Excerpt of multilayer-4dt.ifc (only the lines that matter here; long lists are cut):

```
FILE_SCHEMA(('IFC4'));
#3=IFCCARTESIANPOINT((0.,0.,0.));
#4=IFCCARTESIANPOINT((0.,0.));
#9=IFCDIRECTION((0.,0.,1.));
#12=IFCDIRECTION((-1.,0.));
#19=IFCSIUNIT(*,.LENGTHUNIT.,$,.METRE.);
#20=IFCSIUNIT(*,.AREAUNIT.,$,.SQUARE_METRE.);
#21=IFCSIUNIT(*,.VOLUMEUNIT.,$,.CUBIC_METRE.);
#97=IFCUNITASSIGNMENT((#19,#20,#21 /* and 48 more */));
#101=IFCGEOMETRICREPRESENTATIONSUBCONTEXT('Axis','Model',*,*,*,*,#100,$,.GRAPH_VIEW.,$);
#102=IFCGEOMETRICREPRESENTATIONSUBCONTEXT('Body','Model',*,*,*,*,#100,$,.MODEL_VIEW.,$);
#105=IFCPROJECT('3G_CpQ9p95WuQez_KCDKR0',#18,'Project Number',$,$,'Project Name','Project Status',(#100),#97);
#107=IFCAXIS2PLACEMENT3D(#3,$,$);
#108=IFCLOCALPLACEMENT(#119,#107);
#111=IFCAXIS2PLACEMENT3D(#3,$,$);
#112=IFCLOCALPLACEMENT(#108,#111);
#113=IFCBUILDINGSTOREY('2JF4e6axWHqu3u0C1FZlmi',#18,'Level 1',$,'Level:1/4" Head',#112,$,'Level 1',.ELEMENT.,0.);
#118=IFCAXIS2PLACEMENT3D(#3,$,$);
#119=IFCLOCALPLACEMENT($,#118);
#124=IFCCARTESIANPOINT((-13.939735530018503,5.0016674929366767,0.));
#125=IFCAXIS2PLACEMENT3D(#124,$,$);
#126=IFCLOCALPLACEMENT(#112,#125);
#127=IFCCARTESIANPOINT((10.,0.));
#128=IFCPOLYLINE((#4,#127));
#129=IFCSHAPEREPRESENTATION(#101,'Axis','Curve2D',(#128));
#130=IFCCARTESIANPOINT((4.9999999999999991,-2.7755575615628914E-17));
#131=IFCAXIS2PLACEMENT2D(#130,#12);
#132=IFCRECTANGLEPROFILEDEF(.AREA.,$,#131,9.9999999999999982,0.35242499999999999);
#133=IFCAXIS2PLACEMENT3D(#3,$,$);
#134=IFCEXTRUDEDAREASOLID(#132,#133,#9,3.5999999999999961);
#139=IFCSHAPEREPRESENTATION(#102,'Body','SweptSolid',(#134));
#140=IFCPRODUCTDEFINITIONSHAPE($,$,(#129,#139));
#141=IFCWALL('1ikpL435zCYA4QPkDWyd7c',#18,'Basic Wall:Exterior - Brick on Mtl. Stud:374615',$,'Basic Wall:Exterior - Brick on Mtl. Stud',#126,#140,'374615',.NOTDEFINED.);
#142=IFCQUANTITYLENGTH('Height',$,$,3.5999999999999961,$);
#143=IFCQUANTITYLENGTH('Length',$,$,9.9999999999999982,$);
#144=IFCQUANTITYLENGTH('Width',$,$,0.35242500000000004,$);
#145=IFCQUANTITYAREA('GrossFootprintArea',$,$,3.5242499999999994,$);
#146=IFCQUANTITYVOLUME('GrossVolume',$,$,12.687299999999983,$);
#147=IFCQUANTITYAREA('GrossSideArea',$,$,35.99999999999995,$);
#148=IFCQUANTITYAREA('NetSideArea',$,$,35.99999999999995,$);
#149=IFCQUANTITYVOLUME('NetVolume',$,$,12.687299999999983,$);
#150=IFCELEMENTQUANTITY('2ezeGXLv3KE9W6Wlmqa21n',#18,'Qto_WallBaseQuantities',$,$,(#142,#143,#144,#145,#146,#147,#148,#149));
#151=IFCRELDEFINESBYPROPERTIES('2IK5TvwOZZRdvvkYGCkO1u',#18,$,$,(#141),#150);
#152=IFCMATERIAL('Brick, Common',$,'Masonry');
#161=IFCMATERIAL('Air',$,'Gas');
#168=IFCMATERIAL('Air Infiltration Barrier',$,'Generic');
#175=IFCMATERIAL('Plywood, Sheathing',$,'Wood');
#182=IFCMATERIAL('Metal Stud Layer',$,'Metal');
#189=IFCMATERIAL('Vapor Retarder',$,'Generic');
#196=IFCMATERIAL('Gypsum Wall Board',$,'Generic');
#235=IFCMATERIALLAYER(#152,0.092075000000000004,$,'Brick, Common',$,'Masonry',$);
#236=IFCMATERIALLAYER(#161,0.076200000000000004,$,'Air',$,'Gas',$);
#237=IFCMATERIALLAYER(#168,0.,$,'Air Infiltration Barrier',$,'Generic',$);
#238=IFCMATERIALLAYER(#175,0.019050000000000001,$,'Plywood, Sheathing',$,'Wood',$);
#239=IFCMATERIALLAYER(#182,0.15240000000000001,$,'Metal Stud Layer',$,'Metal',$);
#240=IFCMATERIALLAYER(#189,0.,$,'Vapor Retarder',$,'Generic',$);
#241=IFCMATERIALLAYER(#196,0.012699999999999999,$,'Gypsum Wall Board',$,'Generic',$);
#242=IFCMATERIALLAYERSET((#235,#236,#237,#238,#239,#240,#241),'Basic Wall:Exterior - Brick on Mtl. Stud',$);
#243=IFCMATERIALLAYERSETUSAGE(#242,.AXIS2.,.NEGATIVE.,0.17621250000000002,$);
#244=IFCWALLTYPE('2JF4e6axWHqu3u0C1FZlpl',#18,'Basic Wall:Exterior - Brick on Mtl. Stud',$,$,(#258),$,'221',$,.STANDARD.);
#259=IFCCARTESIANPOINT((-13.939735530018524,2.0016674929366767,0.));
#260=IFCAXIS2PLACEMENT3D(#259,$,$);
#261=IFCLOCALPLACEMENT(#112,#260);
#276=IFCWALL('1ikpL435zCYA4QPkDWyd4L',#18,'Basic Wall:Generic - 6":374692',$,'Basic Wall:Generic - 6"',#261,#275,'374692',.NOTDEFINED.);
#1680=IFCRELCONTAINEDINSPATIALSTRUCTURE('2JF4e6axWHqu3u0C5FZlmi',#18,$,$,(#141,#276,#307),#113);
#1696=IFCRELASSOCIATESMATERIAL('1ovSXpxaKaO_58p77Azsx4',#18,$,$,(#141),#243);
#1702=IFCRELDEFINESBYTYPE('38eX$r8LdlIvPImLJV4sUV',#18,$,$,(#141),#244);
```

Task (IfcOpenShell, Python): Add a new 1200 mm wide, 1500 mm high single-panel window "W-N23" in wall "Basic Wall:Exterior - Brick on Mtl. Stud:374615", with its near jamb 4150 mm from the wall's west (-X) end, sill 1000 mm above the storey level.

```python
import numpy as np
import ifcopenshell
import ifcopenshell.api.feature
import ifcopenshell.api.geometry
import ifcopenshell.api.pset
import ifcopenshell.api.root
import ifcopenshell.api.spatial
import ifcopenshell.geom
import ifcopenshell.util.element
import ifcopenshell.util.placement
import ifcopenshell.util.representation
import ifcopenshell.util.shape
import ifcopenshell.util.unit

model = ifcopenshell.open("multilayer-4dt.ifc")
unit_scale = ifcopenshell.util.unit.calculate_unit_scale(model)
area_scale = ifcopenshell.util.unit.calculate_unit_scale(model, "AREAUNIT")
volume_scale = ifcopenshell.util.unit.calculate_unit_scale(model, "VOLUMEUNIT")
settings = ifcopenshell.geom.settings()


def volume(element):
    """Net volume in cubic metres, openings subtracted."""
    shape = ifcopenshell.geom.create_shape(settings, element)
    return ifcopenshell.util.shape.get_volume(shape.geometry)


wall = model.by_id(141)
storey = ifcopenshell.util.element.get_container(wall, ifc_class="IfcBuildingStorey")
context = ifcopenshell.util.representation.get_context(model, "Model", "Body", "MODEL_VIEW")
before = volume(wall)

width, height, from_end, sill = 1.2, 1.5, 4.15, 1  # metres

# The wall runs along its own X axis, and the end named is its -X end.
wall_shape = ifcopenshell.geom.create_shape(settings, wall)
x, y, z = ifcopenshell.util.shape.get_vertices(wall_shape.geometry).T
start = x.min() + from_end
face, thickness = float(y.min()), float(y.max() - y.min())
wall_matrix = ifcopenshell.util.placement.get_local_placement(wall.ObjectPlacement)
level = ifcopenshell.util.placement.get_local_placement(storey.ObjectPlacement)[2, 3]


def in_wall(x, y):
    """Placement at x, y metres in the wall's axes, at sill height."""
    matrix = wall_matrix.copy()
    matrix[:, 3] = wall_matrix @ np.array([x / unit_scale, y / unit_scale, 0.0, 1.0])
    matrix[2, 3] = level + sill / unit_scale
    return matrix


# Opening: a box that overshoots both wall faces by 50 mm.
opening = ifcopenshell.api.root.create_entity(model, ifc_class="IfcOpeningElement", predefined_type="OPENING")
box = ifcopenshell.api.geometry.add_wall_representation(
    model, context=context, length=width, height=height, thickness=thickness + 0.1
)
ifcopenshell.api.geometry.assign_representation(model, product=opening, representation=box)
ifcopenshell.api.geometry.edit_object_placement(model, product=opening, matrix=in_wall(start, face - 0.05), is_si=False)
ifcopenshell.api.feature.add_feature(model, feature=opening, element=wall)

window = ifcopenshell.api.root.create_entity(model, ifc_class="IfcWindow", name="W-N23", predefined_type="WINDOW")
window.OverallWidth, window.OverallHeight = width / unit_scale, height / unit_scale
window.PartitioningType = "SINGLE_PANEL"
body = ifcopenshell.api.geometry.add_window_representation(
    model,
    context=context,
    overall_width=window.OverallWidth,
    overall_height=window.OverallHeight,
    partition_type="SINGLE_PANEL",
)
ifcopenshell.api.geometry.assign_representation(model, product=window, representation=body)
ifcopenshell.api.spatial.assign_container(model, products=[window], relating_structure=storey)
ifcopenshell.api.feature.add_filling(model, opening=opening, element=window)

# Centre the window in the wall's thickness.
ifcopenshell.api.geometry.edit_object_placement(model, product=window, matrix=in_wall(start, face), is_si=False)
window_shape = ifcopenshell.geom.create_shape(settings, window)
depth = ifcopenshell.util.shape.get_vertices(window_shape.geometry)[:, 1]
offset = face + thickness / 2 - (depth.min() + depth.max()) / 2
ifcopenshell.api.geometry.edit_object_placement(model, product=window, matrix=in_wall(start, offset), is_si=False)

after = volume(wall)

# Update the wall's stored quantities.
qto = model.by_id(ifcopenshell.util.element.get_pset(wall, "Qto_WallBaseQuantities", should_inherit=False)["id"])
ifcopenshell.api.pset.edit_qto(model, qto=qto, properties={
    "NetSideArea": after / thickness / area_scale,
    "NetVolume": after / volume_scale,
})

print(f"wall volume {before:.3f} -> {after:.3f} m3")

model.write("multilayer-4dt_updated.ifc")
```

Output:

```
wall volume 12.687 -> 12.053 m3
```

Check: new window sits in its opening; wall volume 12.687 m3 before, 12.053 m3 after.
